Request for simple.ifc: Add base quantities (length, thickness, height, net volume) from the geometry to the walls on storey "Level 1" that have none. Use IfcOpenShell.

First a look at what the model holds.

```python
import ifcopenshell
import ifcopenshell.util.element
import ifcopenshell.util.unit

model = ifcopenshell.open("simple.ifc")
print(model.schema)
for unit_type in ("LENGTHUNIT", "AREAUNIT", "VOLUMEUNIT"):
    print(unit_type, ifcopenshell.util.unit.calculate_unit_scale(model, unit_type))
storey = next(s for s in model.by_type("IfcBuildingStorey") if s.Name == "Level 1")
walls = [e for e in ifcopenshell.util.element.get_decomposition(storey) if e.is_a("IfcWall")]
for e in sorted(walls, key=lambda e: e.id()):
    print(e.id(), e.is_a(), e.Name, list(ifcopenshell.util.element.get_psets(e, qtos_only=True)), sep=" | ")
```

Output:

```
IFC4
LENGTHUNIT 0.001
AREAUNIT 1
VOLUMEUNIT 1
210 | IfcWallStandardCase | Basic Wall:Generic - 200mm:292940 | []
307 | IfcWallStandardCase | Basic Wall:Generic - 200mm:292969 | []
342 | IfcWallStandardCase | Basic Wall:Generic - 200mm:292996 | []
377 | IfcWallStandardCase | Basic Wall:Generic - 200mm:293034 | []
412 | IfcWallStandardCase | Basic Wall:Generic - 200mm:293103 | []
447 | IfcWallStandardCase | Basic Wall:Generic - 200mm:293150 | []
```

```python
import ifcopenshell
import ifcopenshell.api.pset
import ifcopenshell.geom
import ifcopenshell.util.element
import ifcopenshell.util.shape
import ifcopenshell.util.unit

model = ifcopenshell.open("simple.ifc")
unit_scale = ifcopenshell.util.unit.calculate_unit_scale(model)
volume_scale = ifcopenshell.util.unit.calculate_unit_scale(model, "VOLUMEUNIT")
settings = ifcopenshell.geom.settings()

storey = next(s for s in model.by_type("IfcBuildingStorey") if s.Name == "Level 1")
walls = [e for e in ifcopenshell.util.element.get_decomposition(storey) if e.is_a("IfcWall")]

for e in sorted(walls, key=lambda e: e.id()):
    if ifcopenshell.util.element.get_psets(e, qtos_only=True, should_inherit=False):
        continue
    # Geometry comes back in metres, in the element's own axes.
    shape = ifcopenshell.geom.create_shape(settings, e)
    values = {
        "Length": ifcopenshell.util.shape.get_x(shape.geometry) / unit_scale,
        "Width": ifcopenshell.util.shape.get_y(shape.geometry) / unit_scale,
        "Height": ifcopenshell.util.shape.get_z(shape.geometry) / unit_scale,
        "NetVolume": ifcopenshell.util.shape.get_volume(shape.geometry) / volume_scale,
    }
    qto = ifcopenshell.api.pset.add_qto(model, product=e, name="Qto_WallBaseQuantities")
    ifcopenshell.api.pset.edit_qto(model, qto=qto, properties=values)
    print(e.id(), {k: round(v, 3) for k, v in values.items()})

model.write("simple_v2.ifc")
```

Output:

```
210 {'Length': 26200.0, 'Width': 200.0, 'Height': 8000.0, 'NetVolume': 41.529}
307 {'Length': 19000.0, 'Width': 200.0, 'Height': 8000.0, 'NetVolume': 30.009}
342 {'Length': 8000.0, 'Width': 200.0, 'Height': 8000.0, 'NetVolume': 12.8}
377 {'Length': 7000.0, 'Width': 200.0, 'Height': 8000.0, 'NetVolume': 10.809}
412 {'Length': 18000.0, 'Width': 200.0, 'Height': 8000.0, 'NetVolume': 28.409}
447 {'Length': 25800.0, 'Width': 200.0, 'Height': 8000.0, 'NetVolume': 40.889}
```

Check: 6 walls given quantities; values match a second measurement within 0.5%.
